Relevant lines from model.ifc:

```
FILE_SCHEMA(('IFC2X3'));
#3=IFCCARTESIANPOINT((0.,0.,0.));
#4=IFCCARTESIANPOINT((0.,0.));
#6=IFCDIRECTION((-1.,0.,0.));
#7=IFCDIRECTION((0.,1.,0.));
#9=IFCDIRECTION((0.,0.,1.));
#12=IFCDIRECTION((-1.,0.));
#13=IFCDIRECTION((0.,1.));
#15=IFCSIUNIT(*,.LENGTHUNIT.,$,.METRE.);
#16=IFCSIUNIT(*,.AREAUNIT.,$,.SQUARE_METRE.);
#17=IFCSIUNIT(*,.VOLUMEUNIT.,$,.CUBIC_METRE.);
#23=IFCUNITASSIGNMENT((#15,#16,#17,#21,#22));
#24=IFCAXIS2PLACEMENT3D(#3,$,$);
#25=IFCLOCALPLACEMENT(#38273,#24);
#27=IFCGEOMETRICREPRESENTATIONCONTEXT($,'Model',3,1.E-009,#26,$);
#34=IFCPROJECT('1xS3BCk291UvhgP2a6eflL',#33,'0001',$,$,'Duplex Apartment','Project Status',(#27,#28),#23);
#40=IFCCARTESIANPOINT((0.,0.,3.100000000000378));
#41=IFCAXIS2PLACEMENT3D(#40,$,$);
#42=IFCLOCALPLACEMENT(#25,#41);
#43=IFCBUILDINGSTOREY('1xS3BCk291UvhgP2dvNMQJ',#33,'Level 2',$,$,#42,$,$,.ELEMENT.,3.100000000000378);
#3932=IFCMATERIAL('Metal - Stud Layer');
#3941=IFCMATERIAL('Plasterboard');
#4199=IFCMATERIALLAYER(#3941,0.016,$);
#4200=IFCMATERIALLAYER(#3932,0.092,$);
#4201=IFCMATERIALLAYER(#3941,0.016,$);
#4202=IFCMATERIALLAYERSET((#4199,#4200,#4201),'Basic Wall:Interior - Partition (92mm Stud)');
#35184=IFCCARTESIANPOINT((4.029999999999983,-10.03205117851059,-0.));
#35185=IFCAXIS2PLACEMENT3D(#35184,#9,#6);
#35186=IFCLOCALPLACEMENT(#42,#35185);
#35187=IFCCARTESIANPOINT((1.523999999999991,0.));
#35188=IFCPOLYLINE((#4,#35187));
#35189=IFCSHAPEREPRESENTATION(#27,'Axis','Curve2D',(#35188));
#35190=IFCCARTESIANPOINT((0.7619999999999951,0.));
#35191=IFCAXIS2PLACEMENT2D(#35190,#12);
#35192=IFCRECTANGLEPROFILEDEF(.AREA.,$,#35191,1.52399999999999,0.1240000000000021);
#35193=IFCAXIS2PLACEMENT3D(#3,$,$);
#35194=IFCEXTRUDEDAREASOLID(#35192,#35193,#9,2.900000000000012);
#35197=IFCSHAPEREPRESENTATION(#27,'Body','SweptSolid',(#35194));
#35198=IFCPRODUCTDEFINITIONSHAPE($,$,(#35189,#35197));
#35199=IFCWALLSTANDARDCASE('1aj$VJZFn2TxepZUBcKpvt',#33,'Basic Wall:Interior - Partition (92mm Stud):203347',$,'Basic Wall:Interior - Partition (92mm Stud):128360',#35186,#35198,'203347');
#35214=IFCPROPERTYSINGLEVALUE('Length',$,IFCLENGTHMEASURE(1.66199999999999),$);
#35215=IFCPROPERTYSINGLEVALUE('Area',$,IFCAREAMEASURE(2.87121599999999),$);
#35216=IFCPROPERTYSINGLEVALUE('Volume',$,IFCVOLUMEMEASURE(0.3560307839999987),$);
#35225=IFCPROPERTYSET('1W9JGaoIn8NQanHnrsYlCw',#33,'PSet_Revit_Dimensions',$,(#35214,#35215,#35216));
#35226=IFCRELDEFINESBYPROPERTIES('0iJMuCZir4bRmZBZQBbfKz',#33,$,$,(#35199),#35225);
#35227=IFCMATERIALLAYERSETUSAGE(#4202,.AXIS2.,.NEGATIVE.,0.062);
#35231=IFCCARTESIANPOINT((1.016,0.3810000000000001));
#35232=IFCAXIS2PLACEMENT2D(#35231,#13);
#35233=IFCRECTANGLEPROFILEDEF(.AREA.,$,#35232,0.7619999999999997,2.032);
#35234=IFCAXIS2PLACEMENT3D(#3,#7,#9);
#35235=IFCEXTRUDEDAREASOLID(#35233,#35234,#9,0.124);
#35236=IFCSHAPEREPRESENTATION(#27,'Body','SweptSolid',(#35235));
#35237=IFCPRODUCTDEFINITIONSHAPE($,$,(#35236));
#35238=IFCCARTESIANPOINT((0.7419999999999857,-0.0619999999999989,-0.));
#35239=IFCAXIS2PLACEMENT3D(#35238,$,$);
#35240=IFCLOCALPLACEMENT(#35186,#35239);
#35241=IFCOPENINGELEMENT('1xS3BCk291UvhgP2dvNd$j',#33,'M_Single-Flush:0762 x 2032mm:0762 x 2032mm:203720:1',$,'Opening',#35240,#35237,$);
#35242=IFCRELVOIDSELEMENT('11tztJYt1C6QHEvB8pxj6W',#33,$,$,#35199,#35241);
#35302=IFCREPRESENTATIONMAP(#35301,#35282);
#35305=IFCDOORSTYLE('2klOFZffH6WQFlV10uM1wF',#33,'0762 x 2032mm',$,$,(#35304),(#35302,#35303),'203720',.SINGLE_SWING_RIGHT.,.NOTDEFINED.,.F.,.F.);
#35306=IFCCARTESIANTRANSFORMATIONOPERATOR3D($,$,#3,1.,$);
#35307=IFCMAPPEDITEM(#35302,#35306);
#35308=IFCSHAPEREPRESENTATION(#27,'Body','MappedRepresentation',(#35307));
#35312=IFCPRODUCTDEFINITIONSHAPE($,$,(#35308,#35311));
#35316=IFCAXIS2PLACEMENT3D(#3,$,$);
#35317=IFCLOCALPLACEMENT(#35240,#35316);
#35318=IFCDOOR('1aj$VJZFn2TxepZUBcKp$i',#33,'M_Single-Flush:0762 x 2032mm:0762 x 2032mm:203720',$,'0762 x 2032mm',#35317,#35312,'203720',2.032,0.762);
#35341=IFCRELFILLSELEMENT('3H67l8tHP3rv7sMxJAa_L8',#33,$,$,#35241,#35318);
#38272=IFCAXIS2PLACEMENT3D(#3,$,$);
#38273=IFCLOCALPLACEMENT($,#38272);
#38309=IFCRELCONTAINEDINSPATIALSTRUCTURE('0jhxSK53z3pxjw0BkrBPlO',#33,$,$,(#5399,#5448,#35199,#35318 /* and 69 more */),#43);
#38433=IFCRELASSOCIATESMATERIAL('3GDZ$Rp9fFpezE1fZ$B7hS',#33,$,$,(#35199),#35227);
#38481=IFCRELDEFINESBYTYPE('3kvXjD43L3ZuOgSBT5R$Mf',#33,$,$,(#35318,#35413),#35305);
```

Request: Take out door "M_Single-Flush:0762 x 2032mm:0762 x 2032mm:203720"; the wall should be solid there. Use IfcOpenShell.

```python
import ifcopenshell
import ifcopenshell.api.feature
import ifcopenshell.api.pset
import ifcopenshell.api.root
import ifcopenshell.geom
import ifcopenshell.util.element
import ifcopenshell.util.shape
import ifcopenshell.util.unit

model = ifcopenshell.open("model.ifc")
area_scale = ifcopenshell.util.unit.calculate_unit_scale(model, "AREAUNIT")
volume_scale = ifcopenshell.util.unit.calculate_unit_scale(model, "VOLUMEUNIT")
settings = ifcopenshell.geom.settings()


def volume(element):
    """Net volume in cubic metres, openings subtracted."""
    shape = ifcopenshell.geom.create_shape(settings, element)
    return ifcopenshell.util.shape.get_volume(shape.geometry)


door = model.by_guid("1aj$VJZFn2TxepZUBcKp$i")
opening = door.FillsVoids[0].RelatingOpeningElement
wall = opening.VoidsElements[0].RelatingBuildingElement
before = volume(wall)

ifcopenshell.api.root.remove_product(model, product=door)
ifcopenshell.api.feature.remove_feature(model, feature=opening)

after = volume(wall)
thickness = 0.124  # wall thickness in metres

# Update the wall's stored quantities.
pset = model.by_id(ifcopenshell.util.element.get_pset(wall, "PSet_Revit_Dimensions", should_inherit=False)["id"])
ifcopenshell.api.pset.edit_pset(model, pset=pset, properties={
    "Area": model.create_entity("IfcAreaMeasure", after / thickness / area_scale),
    "Volume": model.create_entity("IfcVolumeMeasure", after / volume_scale),
})

print(f"wall volume {before:.3f} -> {after:.3f} m3")

model.write("model-out.ifc")
```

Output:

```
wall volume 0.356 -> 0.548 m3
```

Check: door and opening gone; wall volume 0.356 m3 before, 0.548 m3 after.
